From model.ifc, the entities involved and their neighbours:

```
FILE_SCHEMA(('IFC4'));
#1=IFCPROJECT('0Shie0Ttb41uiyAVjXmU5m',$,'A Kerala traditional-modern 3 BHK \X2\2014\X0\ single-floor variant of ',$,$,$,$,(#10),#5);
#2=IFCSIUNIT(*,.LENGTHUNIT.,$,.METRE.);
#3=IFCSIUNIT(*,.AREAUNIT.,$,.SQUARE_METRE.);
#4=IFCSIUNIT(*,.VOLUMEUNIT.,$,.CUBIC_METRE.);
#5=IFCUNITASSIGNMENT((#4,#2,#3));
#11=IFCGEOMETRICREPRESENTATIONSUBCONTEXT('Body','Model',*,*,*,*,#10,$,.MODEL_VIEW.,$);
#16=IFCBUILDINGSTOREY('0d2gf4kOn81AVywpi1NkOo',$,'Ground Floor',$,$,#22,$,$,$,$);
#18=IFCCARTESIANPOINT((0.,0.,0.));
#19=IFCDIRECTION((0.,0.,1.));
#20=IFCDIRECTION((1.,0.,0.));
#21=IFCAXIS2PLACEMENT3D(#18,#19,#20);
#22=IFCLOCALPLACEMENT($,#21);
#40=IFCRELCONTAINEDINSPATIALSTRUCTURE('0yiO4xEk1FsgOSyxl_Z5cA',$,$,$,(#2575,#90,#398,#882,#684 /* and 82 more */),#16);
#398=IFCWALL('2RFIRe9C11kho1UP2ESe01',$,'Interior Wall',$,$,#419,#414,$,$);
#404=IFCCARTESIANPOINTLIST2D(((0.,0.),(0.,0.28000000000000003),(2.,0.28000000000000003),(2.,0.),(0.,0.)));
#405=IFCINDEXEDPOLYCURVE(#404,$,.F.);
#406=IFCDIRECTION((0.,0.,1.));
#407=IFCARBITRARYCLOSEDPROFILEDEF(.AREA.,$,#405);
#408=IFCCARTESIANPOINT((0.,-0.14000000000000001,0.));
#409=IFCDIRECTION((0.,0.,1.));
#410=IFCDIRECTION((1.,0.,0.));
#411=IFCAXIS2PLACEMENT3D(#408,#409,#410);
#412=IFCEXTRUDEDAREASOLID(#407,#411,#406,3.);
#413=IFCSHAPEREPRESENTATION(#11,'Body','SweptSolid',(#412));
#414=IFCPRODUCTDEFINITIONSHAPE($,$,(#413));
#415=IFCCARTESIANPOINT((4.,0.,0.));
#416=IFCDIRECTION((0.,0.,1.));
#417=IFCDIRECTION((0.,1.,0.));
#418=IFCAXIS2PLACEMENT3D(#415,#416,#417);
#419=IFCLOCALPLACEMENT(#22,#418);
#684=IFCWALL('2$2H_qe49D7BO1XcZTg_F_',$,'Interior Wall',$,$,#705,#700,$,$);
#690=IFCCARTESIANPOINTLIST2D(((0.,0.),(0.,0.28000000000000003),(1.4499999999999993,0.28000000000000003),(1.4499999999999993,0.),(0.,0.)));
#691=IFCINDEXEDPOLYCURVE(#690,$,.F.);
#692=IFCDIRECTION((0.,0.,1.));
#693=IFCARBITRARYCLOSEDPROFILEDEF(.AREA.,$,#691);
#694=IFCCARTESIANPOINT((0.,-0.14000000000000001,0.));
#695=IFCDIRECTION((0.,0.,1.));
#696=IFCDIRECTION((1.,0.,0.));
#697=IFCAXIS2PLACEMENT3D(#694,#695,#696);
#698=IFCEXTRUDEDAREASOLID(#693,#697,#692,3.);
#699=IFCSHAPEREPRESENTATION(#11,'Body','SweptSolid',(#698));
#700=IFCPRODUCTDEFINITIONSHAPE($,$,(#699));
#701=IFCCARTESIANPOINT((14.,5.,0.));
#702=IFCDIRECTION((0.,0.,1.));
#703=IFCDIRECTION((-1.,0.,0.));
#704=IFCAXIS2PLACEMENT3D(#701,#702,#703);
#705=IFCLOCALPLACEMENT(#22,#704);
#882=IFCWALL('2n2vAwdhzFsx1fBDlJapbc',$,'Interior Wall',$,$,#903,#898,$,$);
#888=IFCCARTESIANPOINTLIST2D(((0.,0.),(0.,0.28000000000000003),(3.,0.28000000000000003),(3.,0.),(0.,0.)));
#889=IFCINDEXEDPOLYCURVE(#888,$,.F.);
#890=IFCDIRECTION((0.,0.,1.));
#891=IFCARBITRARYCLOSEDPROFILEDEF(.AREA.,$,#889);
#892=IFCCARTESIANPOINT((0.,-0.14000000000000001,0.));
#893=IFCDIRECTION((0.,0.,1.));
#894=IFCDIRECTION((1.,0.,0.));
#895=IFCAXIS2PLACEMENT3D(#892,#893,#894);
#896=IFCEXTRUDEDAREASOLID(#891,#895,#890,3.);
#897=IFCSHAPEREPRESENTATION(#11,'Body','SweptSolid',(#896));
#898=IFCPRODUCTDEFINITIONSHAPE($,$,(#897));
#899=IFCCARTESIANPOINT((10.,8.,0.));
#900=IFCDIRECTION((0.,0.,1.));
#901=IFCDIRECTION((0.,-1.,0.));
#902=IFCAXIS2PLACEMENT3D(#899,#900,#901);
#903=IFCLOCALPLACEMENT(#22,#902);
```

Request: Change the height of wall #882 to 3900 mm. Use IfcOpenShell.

```python
import ifcopenshell
import ifcopenshell.geom
import ifcopenshell.util.representation
import ifcopenshell.util.shape

model = ifcopenshell.open("model.ifc")
settings = ifcopenshell.geom.settings()


def volume(element):
    """Net volume in cubic metres, openings subtracted."""
    shape = ifcopenshell.geom.create_shape(settings, element)
    return ifcopenshell.util.shape.get_volume(shape.geometry)


wall = model.by_id(882)
before = volume(wall)

body = ifcopenshell.util.representation.get_representation(wall, "Model", "Body")
solid = body.Items[0]
old_height = solid.Depth
solid.Depth = 3.9
after = volume(wall)

print(f"height {old_height:g} -> {solid.Depth:g}, volume {before:.3f} -> {after:.3f} m3")

model.write("model_edited.ifc")
```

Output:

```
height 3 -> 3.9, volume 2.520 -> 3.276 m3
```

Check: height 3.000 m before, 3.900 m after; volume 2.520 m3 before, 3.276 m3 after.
